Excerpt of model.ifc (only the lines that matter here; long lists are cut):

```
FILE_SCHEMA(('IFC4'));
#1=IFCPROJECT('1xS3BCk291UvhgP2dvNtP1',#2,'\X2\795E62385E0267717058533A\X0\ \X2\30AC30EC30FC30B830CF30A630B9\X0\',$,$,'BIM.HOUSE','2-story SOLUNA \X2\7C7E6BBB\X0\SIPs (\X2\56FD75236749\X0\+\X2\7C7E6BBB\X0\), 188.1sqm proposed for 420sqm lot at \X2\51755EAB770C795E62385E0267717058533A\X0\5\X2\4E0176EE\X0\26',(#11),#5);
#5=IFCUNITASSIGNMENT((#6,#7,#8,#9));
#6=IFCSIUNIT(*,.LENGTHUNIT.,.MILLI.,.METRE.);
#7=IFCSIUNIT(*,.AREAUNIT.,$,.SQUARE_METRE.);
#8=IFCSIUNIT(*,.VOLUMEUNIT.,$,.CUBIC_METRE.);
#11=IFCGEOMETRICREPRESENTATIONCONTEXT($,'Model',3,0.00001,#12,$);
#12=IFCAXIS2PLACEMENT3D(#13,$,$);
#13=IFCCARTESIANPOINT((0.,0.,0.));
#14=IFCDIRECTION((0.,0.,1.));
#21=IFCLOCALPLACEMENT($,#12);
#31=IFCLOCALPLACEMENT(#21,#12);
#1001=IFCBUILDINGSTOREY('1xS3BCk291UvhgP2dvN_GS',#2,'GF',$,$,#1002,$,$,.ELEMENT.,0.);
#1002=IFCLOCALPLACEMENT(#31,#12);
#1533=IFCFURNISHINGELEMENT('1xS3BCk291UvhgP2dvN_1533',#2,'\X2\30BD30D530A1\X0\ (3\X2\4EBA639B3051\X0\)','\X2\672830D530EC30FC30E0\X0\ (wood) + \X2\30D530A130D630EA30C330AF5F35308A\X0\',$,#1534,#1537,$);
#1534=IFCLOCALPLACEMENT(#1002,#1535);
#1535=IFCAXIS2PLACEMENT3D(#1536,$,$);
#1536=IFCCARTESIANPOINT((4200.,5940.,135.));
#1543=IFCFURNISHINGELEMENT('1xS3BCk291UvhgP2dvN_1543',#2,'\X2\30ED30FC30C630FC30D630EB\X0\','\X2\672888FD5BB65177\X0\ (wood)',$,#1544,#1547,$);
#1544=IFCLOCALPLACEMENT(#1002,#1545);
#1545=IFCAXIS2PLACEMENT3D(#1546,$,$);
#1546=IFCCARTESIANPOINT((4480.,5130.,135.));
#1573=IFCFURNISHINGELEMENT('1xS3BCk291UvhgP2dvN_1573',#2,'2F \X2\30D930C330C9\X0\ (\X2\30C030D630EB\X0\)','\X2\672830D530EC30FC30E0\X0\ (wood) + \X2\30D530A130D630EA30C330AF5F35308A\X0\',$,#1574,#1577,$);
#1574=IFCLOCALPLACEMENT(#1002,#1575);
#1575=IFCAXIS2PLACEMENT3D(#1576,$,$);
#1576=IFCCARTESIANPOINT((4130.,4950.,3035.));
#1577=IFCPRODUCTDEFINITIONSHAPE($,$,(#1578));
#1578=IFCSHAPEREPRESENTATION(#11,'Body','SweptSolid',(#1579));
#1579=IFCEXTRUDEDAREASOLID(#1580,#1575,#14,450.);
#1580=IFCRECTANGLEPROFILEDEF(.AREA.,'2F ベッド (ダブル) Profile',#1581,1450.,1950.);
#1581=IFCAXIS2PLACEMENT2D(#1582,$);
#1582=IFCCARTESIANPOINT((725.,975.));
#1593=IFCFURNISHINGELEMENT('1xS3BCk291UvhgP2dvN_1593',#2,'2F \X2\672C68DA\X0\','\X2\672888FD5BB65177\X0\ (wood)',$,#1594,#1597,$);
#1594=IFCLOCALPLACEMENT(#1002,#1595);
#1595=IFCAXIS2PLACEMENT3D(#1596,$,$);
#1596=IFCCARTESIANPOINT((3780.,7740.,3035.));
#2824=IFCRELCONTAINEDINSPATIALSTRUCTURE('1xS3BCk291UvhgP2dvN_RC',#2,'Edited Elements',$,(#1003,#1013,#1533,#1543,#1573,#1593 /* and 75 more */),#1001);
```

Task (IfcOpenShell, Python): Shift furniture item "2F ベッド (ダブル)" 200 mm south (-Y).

```python
import ifcopenshell
import ifcopenshell.api.geometry
import ifcopenshell.util.placement

model = ifcopenshell.open("model.ifc")

item = model.by_guid("1xS3BCk291UvhgP2dvN_1573")
matrix = ifcopenshell.util.placement.get_local_placement(item.ObjectPlacement)
matrix[1, 3] -= 200.0
ifcopenshell.api.geometry.edit_object_placement(model, product=item, matrix=matrix, is_si=False)

print(ifcopenshell.util.placement.get_local_placement(item.ObjectPlacement).round(3) + 0.0)

model.write("model_v2.ifc")
```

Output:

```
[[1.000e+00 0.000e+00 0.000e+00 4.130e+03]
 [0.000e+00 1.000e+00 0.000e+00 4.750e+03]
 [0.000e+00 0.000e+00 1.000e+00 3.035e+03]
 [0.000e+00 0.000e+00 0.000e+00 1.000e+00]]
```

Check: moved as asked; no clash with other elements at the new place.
